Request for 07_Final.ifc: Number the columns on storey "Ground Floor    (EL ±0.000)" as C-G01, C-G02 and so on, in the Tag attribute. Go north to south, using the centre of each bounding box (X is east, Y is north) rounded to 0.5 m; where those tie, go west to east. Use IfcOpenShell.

First a look at what the model holds.

```python
import ifcopenshell
import ifcopenshell.util.element
import ifcopenshell.util.placement

model = ifcopenshell.open("07_Final.ifc")
print(model.schema)
storey = next(s for s in model.by_type("IfcBuildingStorey") if s.Name == "Ground Floor    (EL ±0.000)")
columns = [e for e in ifcopenshell.util.element.get_decomposition(storey) if e.is_a("IfcColumn")]
for e in sorted(columns, key=lambda e: e.id()):
    origin = ifcopenshell.util.placement.get_local_placement(e.ObjectPlacement)[:3, 3]
    print(e.id(), e.Tag, e.Name, origin.round(2) + 0.0, sep=" | ")
```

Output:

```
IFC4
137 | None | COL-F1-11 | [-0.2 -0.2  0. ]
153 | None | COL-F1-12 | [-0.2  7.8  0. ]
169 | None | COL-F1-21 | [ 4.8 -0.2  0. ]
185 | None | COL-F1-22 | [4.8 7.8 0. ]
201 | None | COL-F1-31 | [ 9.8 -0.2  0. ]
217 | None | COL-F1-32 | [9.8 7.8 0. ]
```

```python
import ifcopenshell
import ifcopenshell.geom
import ifcopenshell.util.element
import ifcopenshell.util.shape

model = ifcopenshell.open("07_Final.ifc")
settings = ifcopenshell.geom.settings()
settings.set("use-world-coords", True)


def centre(element):
    shape = ifcopenshell.geom.create_shape(settings, element)
    return ifcopenshell.util.shape.get_bbox_centroid(shape.geometry)


storey = next(s for s in model.by_type("IfcBuildingStorey") if s.Name == "Ground Floor    (EL ±0.000)")
columns = [e for e in ifcopenshell.util.element.get_decomposition(storey) if e.is_a("IfcColumn")]

# Insertion points can sit at a corner or the storey origin, so sort by the geometry (in metres).
centres = {e: centre(e) for e in columns}
columns.sort(key=lambda e: (-round(centres[e][1] / 0.5), centres[e][0]))

for i, e in enumerate(columns, start=1):
    number = f"C-G{i:02d}"
    e.Tag = number
    print(e.id(), number)

model.write("07_Final_edited.ifc")
```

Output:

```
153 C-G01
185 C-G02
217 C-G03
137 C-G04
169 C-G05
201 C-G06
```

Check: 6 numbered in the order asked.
